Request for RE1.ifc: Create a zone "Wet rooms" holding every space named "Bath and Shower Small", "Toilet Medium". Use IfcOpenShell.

First a look at what the model holds.

```python
import ifcopenshell

model = ifcopenshell.open("RE1.ifc")
print(model.schema)
seen = {}
for space in model.by_type("IfcSpace"):
    seen[space.LongName] = seen.get(space.LongName, 0) + 1
for name, count in sorted(seen.items(), key=str):
    print(count, "x", name)
print("zones:", [z.Name for z in model.by_type("IfcZone")][:20])
```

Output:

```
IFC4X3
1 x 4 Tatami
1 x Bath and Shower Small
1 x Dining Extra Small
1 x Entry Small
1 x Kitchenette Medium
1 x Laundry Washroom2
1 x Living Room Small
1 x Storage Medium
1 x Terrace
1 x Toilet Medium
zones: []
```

```python
import ifcopenshell
import ifcopenshell.api.group
import ifcopenshell.api.root

model = ifcopenshell.open("RE1.ifc")

names = {"Bath and Shower Small", "Toilet Medium"}
spaces = [s for s in model.by_type("IfcSpace") if s.LongName in names]

zone = ifcopenshell.api.root.create_entity(model, ifc_class="IfcZone", name="Wet rooms")
ifcopenshell.api.group.assign_group(model, products=spaces, group=zone)
print(len(spaces), "spaces in", zone.Name)

model.write("RE1-out.ifc")
```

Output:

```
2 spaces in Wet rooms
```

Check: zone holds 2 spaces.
